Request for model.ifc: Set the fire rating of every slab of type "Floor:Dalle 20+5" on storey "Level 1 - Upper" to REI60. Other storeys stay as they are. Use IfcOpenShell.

First a look at what the model holds.

```python
import ifcopenshell
import ifcopenshell.util.element

model = ifcopenshell.open("model.ifc")
print(model.schema)
storey = next(s for s in model.by_type("IfcBuildingStorey") if s.Name == "Level 1 - Upper")
slabs = [e for e in ifcopenshell.util.element.get_decomposition(storey) if e.is_a("IfcSlab")]
seen = {}
for e in slabs:
    element_type = ifcopenshell.util.element.get_type(e)
    key = (element_type.Name if element_type != e and element_type else None, ifcopenshell.util.element.get_pset(e, "Pset_SlabCommon", "FireRating"))
    seen[key] = seen.get(key, 0) + 1
for (name, value), count in sorted(seen.items(), key=str):
    print(count, "x", name, "|", value)
```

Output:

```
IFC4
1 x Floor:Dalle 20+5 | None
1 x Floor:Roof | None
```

```python
import ifcopenshell
import ifcopenshell.api.pset
import ifcopenshell.util.element

model = ifcopenshell.open("model.ifc")

storey = next(s for s in model.by_type("IfcBuildingStorey") if s.Name == "Level 1 - Upper")
slabs = [e for e in ifcopenshell.util.element.get_decomposition(storey) if e.is_a("IfcSlab")]

count = 0
for e in slabs:
    element_type = ifcopenshell.util.element.get_type(e)
    if element_type in (None, e) or element_type.Name != "Floor:Dalle 20+5":
        continue
    # add_pset returns the element's existing set when there is one.
    pset = ifcopenshell.api.pset.add_pset(model, product=e, name="Pset_SlabCommon")
    ifcopenshell.api.pset.edit_pset(model, pset=pset, properties={"FireRating": "REI60"})
    count += 1

print(count, "slabs updated")

model.write("model_rev.ifc")
```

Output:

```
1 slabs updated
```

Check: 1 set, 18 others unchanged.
